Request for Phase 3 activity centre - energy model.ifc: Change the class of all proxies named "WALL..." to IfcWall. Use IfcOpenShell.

First a look at what the model holds.

```python
import re

import ifcopenshell

model = ifcopenshell.open("Phase 3 activity centre - energy model.ifc")
print(model.schema)
seen = {}
for e in model.by_type("IfcBuildingElementProxy"):
    name = re.sub(r":\d+(:\d+)?$", "", e.Name or "")  # drop the element id that some exporters append
    seen[name] = seen.get(name, 0) + 1
for name, count in sorted(seen.items()):
    print(count, "x", name)
```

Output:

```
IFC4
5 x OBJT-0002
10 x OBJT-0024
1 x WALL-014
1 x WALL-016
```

```python
import ifcopenshell
import ifcopenshell.api.root

model = ifcopenshell.open("Phase 3 activity centre - energy model.ifc")

proxies = [e.id() for e in model.by_type("IfcBuildingElementProxy") if (e.Name or "").startswith("WALL")]
for step_id in proxies:
    proxy = model.by_id(step_id)
    # Reclassifying a typed element also reclassifies its type and the type's other occurrences.
    if proxy.is_a("IfcBuildingElementProxy"):
        ifcopenshell.api.root.reassign_class(model, product=proxy, ifc_class="IfcWall")

print(sum(model.by_id(i).is_a("IfcWall") for i in proxies), "reclassified")

model.write("Phase 3 activity centre - energy model-out.ifc")
```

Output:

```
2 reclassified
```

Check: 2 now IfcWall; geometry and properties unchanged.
